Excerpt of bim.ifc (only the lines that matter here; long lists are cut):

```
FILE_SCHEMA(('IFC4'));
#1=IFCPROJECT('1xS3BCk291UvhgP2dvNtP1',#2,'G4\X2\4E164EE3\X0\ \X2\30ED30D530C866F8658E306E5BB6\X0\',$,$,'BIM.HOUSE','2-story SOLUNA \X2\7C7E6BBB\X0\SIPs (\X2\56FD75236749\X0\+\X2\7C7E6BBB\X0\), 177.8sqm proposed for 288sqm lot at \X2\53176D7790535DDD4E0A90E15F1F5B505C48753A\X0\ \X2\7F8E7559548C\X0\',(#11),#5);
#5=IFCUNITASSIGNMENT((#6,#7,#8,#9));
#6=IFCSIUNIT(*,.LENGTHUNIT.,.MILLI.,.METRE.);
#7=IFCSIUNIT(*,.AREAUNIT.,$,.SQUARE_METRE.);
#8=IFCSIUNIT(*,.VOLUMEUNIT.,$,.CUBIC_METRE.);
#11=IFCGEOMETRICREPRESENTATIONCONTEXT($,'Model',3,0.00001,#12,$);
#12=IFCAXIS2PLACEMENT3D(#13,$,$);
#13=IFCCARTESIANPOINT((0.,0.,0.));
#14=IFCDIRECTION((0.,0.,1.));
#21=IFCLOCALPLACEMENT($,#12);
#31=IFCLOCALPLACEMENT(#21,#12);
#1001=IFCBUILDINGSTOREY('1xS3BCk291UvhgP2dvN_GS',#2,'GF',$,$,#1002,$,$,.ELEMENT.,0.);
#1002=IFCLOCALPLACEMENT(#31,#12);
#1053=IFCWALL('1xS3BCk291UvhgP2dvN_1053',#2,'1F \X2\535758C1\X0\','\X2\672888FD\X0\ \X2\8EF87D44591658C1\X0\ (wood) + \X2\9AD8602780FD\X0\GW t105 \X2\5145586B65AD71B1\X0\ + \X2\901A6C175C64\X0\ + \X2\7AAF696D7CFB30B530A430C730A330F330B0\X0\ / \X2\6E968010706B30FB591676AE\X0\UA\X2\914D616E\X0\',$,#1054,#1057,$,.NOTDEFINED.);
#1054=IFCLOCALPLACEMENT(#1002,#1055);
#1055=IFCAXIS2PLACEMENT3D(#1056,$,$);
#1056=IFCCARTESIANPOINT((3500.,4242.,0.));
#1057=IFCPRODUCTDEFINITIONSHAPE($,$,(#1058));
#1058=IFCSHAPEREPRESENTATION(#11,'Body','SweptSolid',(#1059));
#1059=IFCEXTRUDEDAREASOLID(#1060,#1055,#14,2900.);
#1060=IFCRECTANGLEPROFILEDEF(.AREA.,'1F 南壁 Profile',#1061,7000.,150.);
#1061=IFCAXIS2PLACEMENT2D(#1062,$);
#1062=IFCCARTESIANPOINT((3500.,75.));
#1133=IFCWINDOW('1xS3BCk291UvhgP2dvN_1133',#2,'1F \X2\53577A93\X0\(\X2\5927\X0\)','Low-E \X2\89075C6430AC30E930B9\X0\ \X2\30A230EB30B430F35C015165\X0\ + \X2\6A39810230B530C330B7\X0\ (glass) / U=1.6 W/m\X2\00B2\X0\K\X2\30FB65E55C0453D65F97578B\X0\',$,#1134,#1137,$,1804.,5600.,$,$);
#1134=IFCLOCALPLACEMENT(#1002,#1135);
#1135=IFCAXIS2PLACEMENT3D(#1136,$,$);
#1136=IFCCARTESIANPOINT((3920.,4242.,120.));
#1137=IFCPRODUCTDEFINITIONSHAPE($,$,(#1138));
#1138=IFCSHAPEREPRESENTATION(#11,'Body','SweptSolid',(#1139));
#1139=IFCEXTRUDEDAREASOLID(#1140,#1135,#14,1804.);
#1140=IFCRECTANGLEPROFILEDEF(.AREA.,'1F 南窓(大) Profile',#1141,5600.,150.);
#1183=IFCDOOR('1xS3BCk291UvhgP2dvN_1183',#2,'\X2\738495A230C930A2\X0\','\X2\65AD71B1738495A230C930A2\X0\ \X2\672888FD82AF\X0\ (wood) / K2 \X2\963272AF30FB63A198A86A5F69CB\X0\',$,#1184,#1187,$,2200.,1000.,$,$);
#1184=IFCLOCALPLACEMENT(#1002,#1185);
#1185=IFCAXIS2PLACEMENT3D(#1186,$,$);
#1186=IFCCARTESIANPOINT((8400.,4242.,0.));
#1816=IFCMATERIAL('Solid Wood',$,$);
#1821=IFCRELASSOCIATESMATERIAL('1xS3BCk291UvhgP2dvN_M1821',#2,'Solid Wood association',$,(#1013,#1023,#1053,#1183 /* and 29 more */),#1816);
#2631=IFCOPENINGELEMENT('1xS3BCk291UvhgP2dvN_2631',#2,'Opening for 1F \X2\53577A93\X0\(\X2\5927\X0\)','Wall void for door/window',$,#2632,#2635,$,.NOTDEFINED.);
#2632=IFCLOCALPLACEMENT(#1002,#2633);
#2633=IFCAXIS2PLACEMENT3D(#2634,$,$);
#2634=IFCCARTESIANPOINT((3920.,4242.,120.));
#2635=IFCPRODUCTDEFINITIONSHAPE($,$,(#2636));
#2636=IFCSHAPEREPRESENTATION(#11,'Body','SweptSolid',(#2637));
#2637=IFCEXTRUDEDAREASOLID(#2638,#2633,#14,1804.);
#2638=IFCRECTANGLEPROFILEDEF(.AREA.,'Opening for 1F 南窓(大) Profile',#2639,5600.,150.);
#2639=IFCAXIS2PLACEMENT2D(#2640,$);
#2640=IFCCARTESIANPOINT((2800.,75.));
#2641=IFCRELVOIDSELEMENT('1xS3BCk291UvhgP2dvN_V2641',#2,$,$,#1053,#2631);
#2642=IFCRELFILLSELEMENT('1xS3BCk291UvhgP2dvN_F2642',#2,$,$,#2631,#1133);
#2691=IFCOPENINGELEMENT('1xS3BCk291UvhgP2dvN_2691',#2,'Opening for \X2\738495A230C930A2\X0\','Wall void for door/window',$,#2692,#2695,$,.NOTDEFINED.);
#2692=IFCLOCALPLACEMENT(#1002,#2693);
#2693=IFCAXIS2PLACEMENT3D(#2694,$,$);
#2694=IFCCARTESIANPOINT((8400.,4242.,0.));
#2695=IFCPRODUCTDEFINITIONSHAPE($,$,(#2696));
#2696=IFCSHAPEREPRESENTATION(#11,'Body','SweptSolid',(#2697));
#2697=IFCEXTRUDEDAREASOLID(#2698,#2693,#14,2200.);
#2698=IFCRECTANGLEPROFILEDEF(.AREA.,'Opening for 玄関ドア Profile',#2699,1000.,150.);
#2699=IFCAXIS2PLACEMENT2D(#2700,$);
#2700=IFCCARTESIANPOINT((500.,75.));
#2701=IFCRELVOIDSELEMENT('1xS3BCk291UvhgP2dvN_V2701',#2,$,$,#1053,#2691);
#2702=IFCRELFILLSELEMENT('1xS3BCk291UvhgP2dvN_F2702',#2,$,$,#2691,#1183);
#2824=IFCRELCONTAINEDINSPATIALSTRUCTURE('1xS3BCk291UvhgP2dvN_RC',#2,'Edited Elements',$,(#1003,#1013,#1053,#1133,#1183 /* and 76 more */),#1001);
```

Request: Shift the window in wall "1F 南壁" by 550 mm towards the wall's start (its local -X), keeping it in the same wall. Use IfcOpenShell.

```python
import ifcopenshell
import ifcopenshell.api.geometry
import ifcopenshell.util.placement
import ifcopenshell.util.unit

model = ifcopenshell.open("bim.ifc")
unit_scale = ifcopenshell.util.unit.calculate_unit_scale(model)

window = model.by_guid("1xS3BCk291UvhgP2dvN_1133")
opening = window.FillsVoids[0].RelatingOpeningElement
wall = opening.VoidsElements[0].RelatingBuildingElement

wall_matrix = ifcopenshell.util.placement.get_local_placement(wall.ObjectPlacement)
shift = wall_matrix[:3, 0] * -0.55 / unit_scale
before = ifcopenshell.util.placement.get_local_placement(window.ObjectPlacement)[:3, 3].copy()

# The window is not placed relative to its opening, so move both.
for product in (opening, window):
    matrix = ifcopenshell.util.placement.get_local_placement(product.ObjectPlacement)
    matrix[:3, 3] += shift
    ifcopenshell.api.geometry.edit_object_placement(model, product=product, matrix=matrix, is_si=False)

after = ifcopenshell.util.placement.get_local_placement(window.ObjectPlacement)[:3, 3]
print("window moved by", (after - before).round(3) + 0.0)

model.write("bim_rev.ifc")
```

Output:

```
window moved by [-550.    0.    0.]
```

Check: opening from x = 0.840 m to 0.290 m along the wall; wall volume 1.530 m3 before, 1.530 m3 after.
